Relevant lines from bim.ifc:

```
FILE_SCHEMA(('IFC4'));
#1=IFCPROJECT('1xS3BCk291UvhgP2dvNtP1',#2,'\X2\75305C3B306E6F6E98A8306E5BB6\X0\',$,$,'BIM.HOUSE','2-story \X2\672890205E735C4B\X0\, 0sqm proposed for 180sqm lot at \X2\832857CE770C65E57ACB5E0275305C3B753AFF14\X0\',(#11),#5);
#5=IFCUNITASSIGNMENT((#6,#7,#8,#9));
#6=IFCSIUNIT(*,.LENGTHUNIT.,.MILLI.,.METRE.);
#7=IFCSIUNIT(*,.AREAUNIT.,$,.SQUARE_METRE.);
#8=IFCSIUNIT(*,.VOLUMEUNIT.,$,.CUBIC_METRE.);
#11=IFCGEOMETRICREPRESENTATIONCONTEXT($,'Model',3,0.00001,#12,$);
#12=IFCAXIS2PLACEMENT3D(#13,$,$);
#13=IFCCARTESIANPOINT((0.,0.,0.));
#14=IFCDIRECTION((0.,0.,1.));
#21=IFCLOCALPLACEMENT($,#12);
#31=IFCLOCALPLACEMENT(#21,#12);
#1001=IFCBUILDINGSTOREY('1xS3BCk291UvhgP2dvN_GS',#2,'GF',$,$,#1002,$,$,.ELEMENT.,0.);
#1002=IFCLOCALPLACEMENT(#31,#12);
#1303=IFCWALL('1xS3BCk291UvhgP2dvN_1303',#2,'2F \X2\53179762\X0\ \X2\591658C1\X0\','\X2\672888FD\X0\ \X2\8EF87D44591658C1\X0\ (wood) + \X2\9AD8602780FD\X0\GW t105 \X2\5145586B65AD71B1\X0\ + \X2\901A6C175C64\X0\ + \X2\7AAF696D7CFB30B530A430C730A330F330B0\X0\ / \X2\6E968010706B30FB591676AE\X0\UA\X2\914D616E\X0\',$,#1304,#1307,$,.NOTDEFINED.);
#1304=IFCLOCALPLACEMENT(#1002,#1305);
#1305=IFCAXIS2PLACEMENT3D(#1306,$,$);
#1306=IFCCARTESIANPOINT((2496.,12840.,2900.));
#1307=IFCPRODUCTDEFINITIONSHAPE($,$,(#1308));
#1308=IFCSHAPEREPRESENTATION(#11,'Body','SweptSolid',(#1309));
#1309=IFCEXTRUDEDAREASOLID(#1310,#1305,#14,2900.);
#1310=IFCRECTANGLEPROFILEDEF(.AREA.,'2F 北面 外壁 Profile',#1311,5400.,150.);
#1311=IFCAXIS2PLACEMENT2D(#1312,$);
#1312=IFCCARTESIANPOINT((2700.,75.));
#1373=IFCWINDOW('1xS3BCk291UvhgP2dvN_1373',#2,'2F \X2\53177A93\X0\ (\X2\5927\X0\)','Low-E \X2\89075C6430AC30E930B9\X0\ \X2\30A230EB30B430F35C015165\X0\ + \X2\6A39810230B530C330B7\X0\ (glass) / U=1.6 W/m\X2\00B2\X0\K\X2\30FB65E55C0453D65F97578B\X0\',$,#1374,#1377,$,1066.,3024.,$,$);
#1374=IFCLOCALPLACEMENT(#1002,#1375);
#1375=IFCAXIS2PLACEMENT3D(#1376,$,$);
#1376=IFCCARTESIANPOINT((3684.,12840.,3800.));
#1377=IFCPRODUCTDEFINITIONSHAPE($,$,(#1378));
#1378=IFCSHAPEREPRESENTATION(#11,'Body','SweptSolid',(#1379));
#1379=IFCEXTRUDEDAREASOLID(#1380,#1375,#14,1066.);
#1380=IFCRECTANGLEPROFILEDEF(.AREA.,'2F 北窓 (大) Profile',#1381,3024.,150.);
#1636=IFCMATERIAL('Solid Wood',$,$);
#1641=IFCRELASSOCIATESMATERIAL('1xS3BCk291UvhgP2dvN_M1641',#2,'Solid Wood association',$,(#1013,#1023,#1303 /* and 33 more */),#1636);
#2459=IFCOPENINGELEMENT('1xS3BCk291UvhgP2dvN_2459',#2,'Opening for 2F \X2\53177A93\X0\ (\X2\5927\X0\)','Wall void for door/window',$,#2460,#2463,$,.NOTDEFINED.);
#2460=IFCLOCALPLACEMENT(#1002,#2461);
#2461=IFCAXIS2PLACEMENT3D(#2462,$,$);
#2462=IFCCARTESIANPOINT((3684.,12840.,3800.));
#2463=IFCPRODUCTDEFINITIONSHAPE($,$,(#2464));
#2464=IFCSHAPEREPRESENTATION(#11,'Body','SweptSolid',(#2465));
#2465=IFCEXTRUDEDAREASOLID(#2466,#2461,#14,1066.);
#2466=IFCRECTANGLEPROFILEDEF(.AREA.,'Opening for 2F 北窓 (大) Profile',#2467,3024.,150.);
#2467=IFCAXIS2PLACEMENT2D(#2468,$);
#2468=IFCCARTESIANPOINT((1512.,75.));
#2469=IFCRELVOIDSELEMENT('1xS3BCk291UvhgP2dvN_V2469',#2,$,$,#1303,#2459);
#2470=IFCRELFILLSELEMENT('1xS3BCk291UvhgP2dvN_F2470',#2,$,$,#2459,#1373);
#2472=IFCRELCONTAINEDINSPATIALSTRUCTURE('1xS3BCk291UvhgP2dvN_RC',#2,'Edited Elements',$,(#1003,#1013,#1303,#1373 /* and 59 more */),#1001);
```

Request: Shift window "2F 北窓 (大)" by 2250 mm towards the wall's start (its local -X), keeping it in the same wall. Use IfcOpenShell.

```python
import ifcopenshell
import ifcopenshell.api.geometry
import ifcopenshell.util.placement
import ifcopenshell.util.unit

model = ifcopenshell.open("bim.ifc")
unit_scale = ifcopenshell.util.unit.calculate_unit_scale(model)

window = model.by_guid("1xS3BCk291UvhgP2dvN_1373")
opening = window.FillsVoids[0].RelatingOpeningElement
wall = opening.VoidsElements[0].RelatingBuildingElement

wall_matrix = ifcopenshell.util.placement.get_local_placement(wall.ObjectPlacement)
shift = wall_matrix[:3, 0] * -2.25 / unit_scale
before = ifcopenshell.util.placement.get_local_placement(window.ObjectPlacement)[:3, 3].copy()

# The window is not placed relative to its opening, so move both.
for product in (opening, window):
    matrix = ifcopenshell.util.placement.get_local_placement(product.ObjectPlacement)
    matrix[:3, 3] += shift
    ifcopenshell.api.geometry.edit_object_placement(model, product=product, matrix=matrix, is_si=False)

after = ifcopenshell.util.placement.get_local_placement(window.ObjectPlacement)[:3, 3]
print("window moved by", (after - before).round(3) + 0.0)

model.write("bim_updated.ifc")
```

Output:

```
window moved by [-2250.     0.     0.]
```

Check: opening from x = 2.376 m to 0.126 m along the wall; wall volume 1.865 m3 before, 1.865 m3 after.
